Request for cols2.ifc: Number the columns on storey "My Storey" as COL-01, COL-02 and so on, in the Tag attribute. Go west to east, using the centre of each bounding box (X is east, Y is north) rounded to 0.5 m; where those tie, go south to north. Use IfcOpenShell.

First a look at what the model holds.

```python
import ifcopenshell
import ifcopenshell.util.element
import ifcopenshell.util.placement

model = ifcopenshell.open("cols2.ifc")
print(model.schema)
storey = next(s for s in model.by_type("IfcBuildingStorey") if s.Name == "My Storey")
columns = [e for e in ifcopenshell.util.element.get_decomposition(storey) if e.is_a("IfcColumn")]
for e in sorted(columns, key=lambda e: e.id()):
    origin = ifcopenshell.util.placement.get_local_placement(e.ObjectPlacement)[:3, 3]
    print(e.id(), e.Tag, e.Name, origin.round(2) + 0.0, sep=" | ")
```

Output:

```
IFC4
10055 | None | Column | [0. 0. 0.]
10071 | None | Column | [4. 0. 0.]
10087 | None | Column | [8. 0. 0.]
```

```python
import ifcopenshell
import ifcopenshell.geom
import ifcopenshell.util.element
import ifcopenshell.util.shape

model = ifcopenshell.open("cols2.ifc")
settings = ifcopenshell.geom.settings()
settings.set("use-world-coords", True)


def centre(element):
    shape = ifcopenshell.geom.create_shape(settings, element)
    return ifcopenshell.util.shape.get_bbox_centroid(shape.geometry)


storey = next(s for s in model.by_type("IfcBuildingStorey") if s.Name == "My Storey")
columns = [e for e in ifcopenshell.util.element.get_decomposition(storey) if e.is_a("IfcColumn")]

# Insertion points can sit at a corner or the storey origin, so sort by the geometry (in metres).
centres = {e: centre(e) for e in columns}
columns.sort(key=lambda e: (round(centres[e][0] / 0.5), centres[e][1]))

for i, e in enumerate(columns, start=1):
    number = f"COL-{i:02d}"
    e.Tag = number
    print(e.id(), number)

model.write("cols2_edited.ifc")
```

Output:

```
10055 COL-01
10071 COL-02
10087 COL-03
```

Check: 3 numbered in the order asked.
